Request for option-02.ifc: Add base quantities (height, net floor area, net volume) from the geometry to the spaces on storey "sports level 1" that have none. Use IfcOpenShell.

First a look at what the model holds.

```python
import ifcopenshell
import ifcopenshell.util.element
import ifcopenshell.util.unit

model = ifcopenshell.open("option-02.ifc")
print(model.schema)
for unit_type in ("LENGTHUNIT", "AREAUNIT", "VOLUMEUNIT"):
    print(unit_type, ifcopenshell.util.unit.calculate_unit_scale(model, unit_type))
storey = next(s for s in model.by_type("IfcBuildingStorey") if s.Name == "sports level 1")
spaces = [e for e in ifcopenshell.util.element.get_decomposition(storey) if e.is_a("IfcSpace")]
for e in sorted(spaces, key=lambda e: e.id()):
    print(e.id(), e.is_a(), e.Name, list(ifcopenshell.util.element.get_psets(e, qtos_only=True)), sep=" | ")
```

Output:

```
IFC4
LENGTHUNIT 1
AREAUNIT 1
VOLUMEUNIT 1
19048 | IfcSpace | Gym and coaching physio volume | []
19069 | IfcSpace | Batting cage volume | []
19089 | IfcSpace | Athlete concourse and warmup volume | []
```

```python
import ifcopenshell
import ifcopenshell.api.pset
import ifcopenshell.geom
import ifcopenshell.util.element
import ifcopenshell.util.shape
import ifcopenshell.util.unit

model = ifcopenshell.open("option-02.ifc")
unit_scale = ifcopenshell.util.unit.calculate_unit_scale(model)
area_scale = ifcopenshell.util.unit.calculate_unit_scale(model, "AREAUNIT")
volume_scale = ifcopenshell.util.unit.calculate_unit_scale(model, "VOLUMEUNIT")
settings = ifcopenshell.geom.settings()

storey = next(s for s in model.by_type("IfcBuildingStorey") if s.Name == "sports level 1")
spaces = [e for e in ifcopenshell.util.element.get_decomposition(storey) if e.is_a("IfcSpace")]

for e in sorted(spaces, key=lambda e: e.id()):
    if ifcopenshell.util.element.get_psets(e, qtos_only=True, should_inherit=False):
        continue
    # Geometry comes back in metres, in the element's own axes.
    shape = ifcopenshell.geom.create_shape(settings, e)
    values = {
        "Height": ifcopenshell.util.shape.get_z(shape.geometry) / unit_scale,
        "NetFloorArea": ifcopenshell.util.shape.get_footprint_area(shape.geometry) / area_scale,
        "NetVolume": ifcopenshell.util.shape.get_volume(shape.geometry) / volume_scale,
    }
    qto = ifcopenshell.api.pset.add_qto(model, product=e, name="Qto_SpaceBaseQuantities")
    ifcopenshell.api.pset.edit_qto(model, qto=qto, properties=values)
    print(e.id(), {k: round(v, 3) for k, v in values.items()})

model.write("option-02_updated.ifc")
```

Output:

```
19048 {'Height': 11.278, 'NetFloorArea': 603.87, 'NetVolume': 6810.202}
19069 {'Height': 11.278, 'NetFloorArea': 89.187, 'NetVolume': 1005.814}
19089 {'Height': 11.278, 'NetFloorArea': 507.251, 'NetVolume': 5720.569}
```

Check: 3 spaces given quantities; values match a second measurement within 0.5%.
